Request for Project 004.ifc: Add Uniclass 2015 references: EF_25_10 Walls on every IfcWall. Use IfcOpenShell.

First a look at what the model holds.

```python
import ifcopenshell

model = ifcopenshell.open("Project 004.ifc")
print(model.schema)
print("classifications:", [c.Name for c in model.by_type("IfcClassification")])
for ifc_class in ("IfcDoor", "IfcRoof", "IfcStair", "IfcWall", "IfcWindow"):
    print(ifc_class, len(model.by_type(ifc_class)))
```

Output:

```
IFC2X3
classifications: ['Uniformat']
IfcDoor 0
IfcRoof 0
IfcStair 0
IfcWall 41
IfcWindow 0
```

```python
import ifcopenshell
import ifcopenshell.api.classification

model = ifcopenshell.open("Project 004.ifc")

# IFC2X3 requires Source and Edition and has no link from the project to the system.
system = model.create_entity("IfcClassification", Source="NBS", Edition="2015", Name="Uniclass 2015")

codes = {
    "IfcWall": ("EF_25_10", "Walls"),
}
for ifc_class, (code, name) in codes.items():
    products = model.by_type(ifc_class)
    ifcopenshell.api.classification.add_reference(
        model, products=products, classification=system, identification=code, name=name
    )
    print(code, len(products))

model.write("Project 004_updated.ifc")
```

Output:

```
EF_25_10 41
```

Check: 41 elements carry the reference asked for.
